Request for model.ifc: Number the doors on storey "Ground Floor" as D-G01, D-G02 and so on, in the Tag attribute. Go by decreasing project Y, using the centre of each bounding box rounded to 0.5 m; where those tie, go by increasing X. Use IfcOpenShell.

First a look at what the model holds.

```python
import ifcopenshell
import ifcopenshell.util.element
import ifcopenshell.util.placement

model = ifcopenshell.open("model.ifc")
print(model.schema)
storey = next(s for s in model.by_type("IfcBuildingStorey") if s.Name == "Ground Floor")
doors = [e for e in ifcopenshell.util.element.get_decomposition(storey) if e.is_a("IfcDoor")]
for e in sorted(doors, key=lambda e: e.id()):
    origin = ifcopenshell.util.placement.get_local_placement(e.ObjectPlacement)[:3, 3]
    print(e.id(), e.Tag, e.Name, origin.round(2) + 0.0, sep=" | ")
```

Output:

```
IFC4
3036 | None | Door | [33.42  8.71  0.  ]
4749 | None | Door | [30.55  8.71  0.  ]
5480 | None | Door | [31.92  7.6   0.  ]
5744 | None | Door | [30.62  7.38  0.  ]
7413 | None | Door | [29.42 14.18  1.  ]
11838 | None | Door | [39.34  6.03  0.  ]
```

```python
import ifcopenshell
import ifcopenshell.geom
import ifcopenshell.util.element
import ifcopenshell.util.shape

model = ifcopenshell.open("model.ifc")
settings = ifcopenshell.geom.settings()
settings.set("use-world-coords", True)


def centre(element):
    shape = ifcopenshell.geom.create_shape(settings, element)
    return ifcopenshell.util.shape.get_bbox_centroid(shape.geometry)


storey = next(s for s in model.by_type("IfcBuildingStorey") if s.Name == "Ground Floor")
doors = [e for e in ifcopenshell.util.element.get_decomposition(storey) if e.is_a("IfcDoor")]

# Insertion points can sit at a corner or the storey origin, so sort by the geometry (in metres).
centres = {e: centre(e) for e in doors}
doors.sort(key=lambda e: (-round(centres[e][1] / 0.5), centres[e][0]))

for i, e in enumerate(doors, start=1):
    number = f"D-G{i:02d}"
    e.Tag = number
    print(e.id(), number)

model.write("model_updated.ifc")
```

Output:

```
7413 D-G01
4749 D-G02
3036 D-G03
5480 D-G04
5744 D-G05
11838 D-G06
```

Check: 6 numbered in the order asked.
